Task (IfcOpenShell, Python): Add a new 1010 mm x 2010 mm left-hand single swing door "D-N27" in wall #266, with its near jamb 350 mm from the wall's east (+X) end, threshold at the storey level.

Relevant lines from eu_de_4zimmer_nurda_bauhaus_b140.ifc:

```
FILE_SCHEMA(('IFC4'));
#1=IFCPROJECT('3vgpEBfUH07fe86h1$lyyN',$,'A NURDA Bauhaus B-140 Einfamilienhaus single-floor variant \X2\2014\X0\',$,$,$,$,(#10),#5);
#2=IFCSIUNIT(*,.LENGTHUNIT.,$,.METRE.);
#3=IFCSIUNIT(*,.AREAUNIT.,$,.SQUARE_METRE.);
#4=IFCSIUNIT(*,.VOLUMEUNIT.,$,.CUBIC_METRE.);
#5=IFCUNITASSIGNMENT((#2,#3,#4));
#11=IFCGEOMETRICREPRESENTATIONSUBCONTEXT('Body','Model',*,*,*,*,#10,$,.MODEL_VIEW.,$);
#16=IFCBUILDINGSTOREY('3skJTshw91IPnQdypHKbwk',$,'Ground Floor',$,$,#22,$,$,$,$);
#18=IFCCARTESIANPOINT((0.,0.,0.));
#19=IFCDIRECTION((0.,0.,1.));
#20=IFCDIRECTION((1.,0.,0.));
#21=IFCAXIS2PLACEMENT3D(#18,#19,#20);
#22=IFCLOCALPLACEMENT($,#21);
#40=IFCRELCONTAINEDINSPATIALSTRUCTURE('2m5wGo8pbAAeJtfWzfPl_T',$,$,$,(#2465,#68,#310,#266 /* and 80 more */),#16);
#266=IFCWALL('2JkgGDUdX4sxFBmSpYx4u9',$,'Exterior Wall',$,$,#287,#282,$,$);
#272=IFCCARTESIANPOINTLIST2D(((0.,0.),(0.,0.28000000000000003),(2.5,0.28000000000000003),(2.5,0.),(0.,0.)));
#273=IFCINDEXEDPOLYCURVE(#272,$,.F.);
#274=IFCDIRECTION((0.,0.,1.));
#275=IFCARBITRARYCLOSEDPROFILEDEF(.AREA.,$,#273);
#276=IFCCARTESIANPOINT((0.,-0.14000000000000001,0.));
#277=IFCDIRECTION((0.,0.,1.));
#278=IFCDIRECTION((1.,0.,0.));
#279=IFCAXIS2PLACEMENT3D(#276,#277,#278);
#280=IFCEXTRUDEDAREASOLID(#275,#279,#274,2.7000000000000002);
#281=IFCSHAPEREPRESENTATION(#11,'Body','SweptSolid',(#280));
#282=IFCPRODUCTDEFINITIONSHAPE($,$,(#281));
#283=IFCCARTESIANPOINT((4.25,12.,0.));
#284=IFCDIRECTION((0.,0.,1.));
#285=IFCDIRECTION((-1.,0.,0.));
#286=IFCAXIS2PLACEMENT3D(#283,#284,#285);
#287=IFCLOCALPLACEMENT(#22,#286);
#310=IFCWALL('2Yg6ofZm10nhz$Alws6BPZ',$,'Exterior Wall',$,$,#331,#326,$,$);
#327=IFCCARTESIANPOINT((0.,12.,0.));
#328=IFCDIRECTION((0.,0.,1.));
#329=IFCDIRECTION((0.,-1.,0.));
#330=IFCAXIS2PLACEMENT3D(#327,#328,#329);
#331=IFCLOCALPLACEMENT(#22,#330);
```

```python
import numpy as np
import ifcopenshell
import ifcopenshell.api.feature
import ifcopenshell.api.geometry
import ifcopenshell.api.root
import ifcopenshell.api.spatial
import ifcopenshell.geom
import ifcopenshell.util.element
import ifcopenshell.util.placement
import ifcopenshell.util.representation
import ifcopenshell.util.shape
import ifcopenshell.util.unit

model = ifcopenshell.open("eu_de_4zimmer_nurda_bauhaus_b140.ifc")
unit_scale = ifcopenshell.util.unit.calculate_unit_scale(model)
settings = ifcopenshell.geom.settings()


def volume(element):
    """Net volume in cubic metres, openings subtracted."""
    shape = ifcopenshell.geom.create_shape(settings, element)
    return ifcopenshell.util.shape.get_volume(shape.geometry)


wall = model.by_guid("2JkgGDUdX4sxFBmSpYx4u9")
storey = ifcopenshell.util.element.get_container(wall, ifc_class="IfcBuildingStorey")
context = ifcopenshell.util.representation.get_context(model, "Model", "Body", "MODEL_VIEW")
before = volume(wall)

width, height, from_end, sill = 1.01, 2.01, 0.35, 0.0  # metres

# The wall runs along its own X axis, and the end named is its -X end.
wall_shape = ifcopenshell.geom.create_shape(settings, wall)
x, y, z = ifcopenshell.util.shape.get_vertices(wall_shape.geometry).T
start = x.min() + from_end
face, thickness = float(y.min()), float(y.max() - y.min())
wall_matrix = ifcopenshell.util.placement.get_local_placement(wall.ObjectPlacement)
level = ifcopenshell.util.placement.get_local_placement(storey.ObjectPlacement)[2, 3]


def in_wall(x, y):
    """Placement at x, y metres in the wall's axes, at sill height."""
    matrix = wall_matrix.copy()
    matrix[:, 3] = wall_matrix @ np.array([x / unit_scale, y / unit_scale, 0.0, 1.0])
    matrix[2, 3] = level + sill / unit_scale
    return matrix


# Opening: a box that overshoots both wall faces by 50 mm.
opening = ifcopenshell.api.root.create_entity(model, ifc_class="IfcOpeningElement", predefined_type="OPENING")
box = ifcopenshell.api.geometry.add_wall_representation(
    model, context=context, length=width, height=height, thickness=thickness + 0.1
)
ifcopenshell.api.geometry.assign_representation(model, product=opening, representation=box)
ifcopenshell.api.geometry.edit_object_placement(model, product=opening, matrix=in_wall(start, face - 0.05), is_si=False)
ifcopenshell.api.feature.add_feature(model, feature=opening, element=wall)

door = ifcopenshell.api.root.create_entity(model, ifc_class="IfcDoor", name="D-N27", predefined_type="DOOR")
door.OverallWidth, door.OverallHeight = width / unit_scale, height / unit_scale
door.OperationType = "SINGLE_SWING_LEFT"
body = ifcopenshell.api.geometry.add_door_representation(
    model,
    context=context,
    overall_width=door.OverallWidth,
    overall_height=door.OverallHeight,
    operation_type="SINGLE_SWING_LEFT",
    lining_properties={"LiningDepth": thickness / unit_scale, "ThresholdDepth": thickness / unit_scale},
)
ifcopenshell.api.geometry.assign_representation(model, product=door, representation=body)
ifcopenshell.api.spatial.assign_container(model, products=[door], relating_structure=storey)
ifcopenshell.api.feature.add_filling(model, opening=opening, element=door)

# The lining spans the wall, so the door starts at the wall face.
ifcopenshell.api.geometry.edit_object_placement(model, product=door, matrix=in_wall(start, face), is_si=False)

after = volume(wall)

print(f"wall volume {before:.3f} -> {after:.3f} m3")

model.write("eu_de_4zimmer_nurda_bauhaus_b140_edited.ifc")
```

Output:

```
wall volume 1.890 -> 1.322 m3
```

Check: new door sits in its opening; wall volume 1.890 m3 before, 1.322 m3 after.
